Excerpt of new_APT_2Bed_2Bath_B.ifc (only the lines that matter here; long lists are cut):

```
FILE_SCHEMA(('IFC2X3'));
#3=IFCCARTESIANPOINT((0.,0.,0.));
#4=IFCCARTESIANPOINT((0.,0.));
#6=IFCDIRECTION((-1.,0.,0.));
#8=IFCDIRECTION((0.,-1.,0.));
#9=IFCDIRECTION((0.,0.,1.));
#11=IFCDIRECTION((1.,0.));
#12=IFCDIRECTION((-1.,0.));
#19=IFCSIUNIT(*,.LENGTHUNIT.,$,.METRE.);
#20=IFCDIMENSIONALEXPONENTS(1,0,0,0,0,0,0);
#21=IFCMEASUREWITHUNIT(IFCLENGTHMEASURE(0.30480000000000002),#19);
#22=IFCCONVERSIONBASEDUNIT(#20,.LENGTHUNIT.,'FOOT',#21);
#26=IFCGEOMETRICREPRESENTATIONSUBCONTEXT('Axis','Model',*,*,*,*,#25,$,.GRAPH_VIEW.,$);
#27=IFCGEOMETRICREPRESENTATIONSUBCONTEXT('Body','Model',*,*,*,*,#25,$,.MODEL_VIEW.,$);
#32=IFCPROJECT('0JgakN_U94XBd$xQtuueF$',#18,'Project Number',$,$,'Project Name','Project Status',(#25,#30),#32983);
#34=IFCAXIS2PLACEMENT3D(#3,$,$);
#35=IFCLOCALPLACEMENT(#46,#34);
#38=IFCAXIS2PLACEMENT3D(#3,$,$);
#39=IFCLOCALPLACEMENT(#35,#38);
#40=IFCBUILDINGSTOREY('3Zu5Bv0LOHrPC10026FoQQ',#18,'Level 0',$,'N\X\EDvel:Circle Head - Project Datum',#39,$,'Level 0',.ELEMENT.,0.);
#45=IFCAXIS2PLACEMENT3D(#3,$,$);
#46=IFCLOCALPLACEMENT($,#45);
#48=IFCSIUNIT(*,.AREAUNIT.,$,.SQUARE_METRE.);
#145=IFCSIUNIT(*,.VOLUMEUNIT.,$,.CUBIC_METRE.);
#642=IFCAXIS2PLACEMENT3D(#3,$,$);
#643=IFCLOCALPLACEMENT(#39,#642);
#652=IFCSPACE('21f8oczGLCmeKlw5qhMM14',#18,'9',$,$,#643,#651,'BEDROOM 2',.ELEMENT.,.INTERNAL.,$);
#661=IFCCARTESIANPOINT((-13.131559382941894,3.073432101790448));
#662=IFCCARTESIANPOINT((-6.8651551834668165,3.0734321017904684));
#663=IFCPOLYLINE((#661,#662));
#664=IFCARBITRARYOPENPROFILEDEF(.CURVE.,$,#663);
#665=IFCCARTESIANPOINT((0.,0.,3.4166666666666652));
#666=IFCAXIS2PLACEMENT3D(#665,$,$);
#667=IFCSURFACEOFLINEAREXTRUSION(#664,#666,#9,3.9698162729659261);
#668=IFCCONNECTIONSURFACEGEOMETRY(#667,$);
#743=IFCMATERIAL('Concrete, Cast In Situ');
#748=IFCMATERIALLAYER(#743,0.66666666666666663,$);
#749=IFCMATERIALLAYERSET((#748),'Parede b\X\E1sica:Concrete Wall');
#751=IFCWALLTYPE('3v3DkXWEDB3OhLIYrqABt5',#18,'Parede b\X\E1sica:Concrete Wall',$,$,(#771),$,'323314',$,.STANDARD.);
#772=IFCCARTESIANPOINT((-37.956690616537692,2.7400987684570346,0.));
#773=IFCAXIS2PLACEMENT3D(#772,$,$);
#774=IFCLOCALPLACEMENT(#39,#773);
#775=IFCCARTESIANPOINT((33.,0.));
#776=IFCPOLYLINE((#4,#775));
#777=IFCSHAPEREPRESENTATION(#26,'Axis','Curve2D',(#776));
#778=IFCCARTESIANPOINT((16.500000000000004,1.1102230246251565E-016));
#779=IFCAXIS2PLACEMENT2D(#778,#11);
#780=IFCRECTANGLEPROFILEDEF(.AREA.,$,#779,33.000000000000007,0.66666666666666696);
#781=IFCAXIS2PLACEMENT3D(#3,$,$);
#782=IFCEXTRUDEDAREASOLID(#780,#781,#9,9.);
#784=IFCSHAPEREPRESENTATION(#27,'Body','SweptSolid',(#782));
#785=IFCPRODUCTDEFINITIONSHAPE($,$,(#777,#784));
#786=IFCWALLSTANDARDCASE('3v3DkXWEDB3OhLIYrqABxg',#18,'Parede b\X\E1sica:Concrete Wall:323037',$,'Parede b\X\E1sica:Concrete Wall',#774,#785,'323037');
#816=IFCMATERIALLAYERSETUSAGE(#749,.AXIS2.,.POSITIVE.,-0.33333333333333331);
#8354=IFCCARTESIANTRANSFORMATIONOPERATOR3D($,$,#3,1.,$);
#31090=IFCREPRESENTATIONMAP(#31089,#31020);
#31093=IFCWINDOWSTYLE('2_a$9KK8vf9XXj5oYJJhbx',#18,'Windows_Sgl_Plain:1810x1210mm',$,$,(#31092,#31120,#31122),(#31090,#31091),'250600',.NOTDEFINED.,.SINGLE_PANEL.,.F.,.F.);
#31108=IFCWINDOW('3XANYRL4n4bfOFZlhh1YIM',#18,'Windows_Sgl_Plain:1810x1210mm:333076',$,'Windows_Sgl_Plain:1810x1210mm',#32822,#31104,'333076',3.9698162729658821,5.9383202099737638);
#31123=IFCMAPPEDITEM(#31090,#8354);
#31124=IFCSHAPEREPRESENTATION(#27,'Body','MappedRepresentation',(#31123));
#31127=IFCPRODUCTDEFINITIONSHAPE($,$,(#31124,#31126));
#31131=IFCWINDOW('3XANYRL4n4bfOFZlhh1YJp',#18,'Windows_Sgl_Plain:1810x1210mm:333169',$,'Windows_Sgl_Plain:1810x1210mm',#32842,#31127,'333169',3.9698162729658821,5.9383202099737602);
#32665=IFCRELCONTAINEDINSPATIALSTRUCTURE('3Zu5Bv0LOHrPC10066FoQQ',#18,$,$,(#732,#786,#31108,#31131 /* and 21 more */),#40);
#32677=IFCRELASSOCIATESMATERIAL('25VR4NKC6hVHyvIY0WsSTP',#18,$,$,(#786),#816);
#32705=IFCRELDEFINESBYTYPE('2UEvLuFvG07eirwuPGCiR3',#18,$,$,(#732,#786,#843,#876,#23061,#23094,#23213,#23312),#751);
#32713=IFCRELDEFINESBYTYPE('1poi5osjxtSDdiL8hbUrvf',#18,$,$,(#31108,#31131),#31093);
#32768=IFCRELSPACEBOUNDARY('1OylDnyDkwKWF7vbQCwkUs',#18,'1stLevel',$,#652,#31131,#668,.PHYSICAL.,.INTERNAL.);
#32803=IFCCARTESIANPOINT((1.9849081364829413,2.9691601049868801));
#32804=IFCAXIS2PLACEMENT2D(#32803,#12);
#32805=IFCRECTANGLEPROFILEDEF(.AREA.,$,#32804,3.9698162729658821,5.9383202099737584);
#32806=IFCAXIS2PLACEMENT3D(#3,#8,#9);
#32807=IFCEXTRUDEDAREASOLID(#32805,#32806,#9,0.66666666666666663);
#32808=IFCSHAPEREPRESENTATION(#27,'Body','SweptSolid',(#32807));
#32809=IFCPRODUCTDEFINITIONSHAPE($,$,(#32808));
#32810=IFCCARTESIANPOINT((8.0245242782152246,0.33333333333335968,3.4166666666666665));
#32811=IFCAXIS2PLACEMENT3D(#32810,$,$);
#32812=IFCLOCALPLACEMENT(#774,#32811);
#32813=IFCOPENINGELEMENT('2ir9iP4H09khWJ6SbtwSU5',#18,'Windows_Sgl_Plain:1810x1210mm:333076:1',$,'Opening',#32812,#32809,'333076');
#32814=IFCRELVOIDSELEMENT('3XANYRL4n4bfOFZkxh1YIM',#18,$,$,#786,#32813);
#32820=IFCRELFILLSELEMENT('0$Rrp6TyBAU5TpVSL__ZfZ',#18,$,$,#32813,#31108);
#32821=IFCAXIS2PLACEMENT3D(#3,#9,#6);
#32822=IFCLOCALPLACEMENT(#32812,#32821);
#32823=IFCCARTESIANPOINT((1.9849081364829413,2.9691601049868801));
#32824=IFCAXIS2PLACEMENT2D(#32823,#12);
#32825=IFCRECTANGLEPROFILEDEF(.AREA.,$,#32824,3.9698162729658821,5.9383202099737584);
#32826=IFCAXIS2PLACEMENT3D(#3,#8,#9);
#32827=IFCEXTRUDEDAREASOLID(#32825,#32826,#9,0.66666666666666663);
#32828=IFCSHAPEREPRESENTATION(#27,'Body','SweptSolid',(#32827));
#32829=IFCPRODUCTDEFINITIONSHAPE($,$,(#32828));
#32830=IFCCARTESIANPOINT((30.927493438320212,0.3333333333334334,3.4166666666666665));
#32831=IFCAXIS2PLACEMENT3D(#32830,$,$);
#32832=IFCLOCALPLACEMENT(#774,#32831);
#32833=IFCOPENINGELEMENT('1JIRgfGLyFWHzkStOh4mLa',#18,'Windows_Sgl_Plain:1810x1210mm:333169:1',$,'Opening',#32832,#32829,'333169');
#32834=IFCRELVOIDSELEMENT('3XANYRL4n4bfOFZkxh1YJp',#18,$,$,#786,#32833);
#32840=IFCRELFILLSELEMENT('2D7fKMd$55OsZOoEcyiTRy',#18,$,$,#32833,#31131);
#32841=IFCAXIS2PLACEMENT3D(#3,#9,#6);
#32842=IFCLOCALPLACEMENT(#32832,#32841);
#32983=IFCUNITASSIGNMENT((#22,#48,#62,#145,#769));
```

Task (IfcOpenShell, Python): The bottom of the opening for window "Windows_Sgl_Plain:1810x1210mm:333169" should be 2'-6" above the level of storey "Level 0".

```python
import numpy as np
import ifcopenshell
import ifcopenshell.api.geometry
import ifcopenshell.geom
import ifcopenshell.util.element
import ifcopenshell.util.placement
import ifcopenshell.util.shape
import ifcopenshell.util.unit

model = ifcopenshell.open("new_APT_2Bed_2Bath_B.ifc")
unit_scale = ifcopenshell.util.unit.calculate_unit_scale(model)

window = model.by_guid("3XANYRL4n4bfOFZlhh1YJp")
opening = window.FillsVoids[0].RelatingOpeningElement
storey = ifcopenshell.util.element.get_container(window, ifc_class="IfcBuildingStorey")
level = ifcopenshell.util.placement.get_local_placement(storey.ObjectPlacement)[2, 3]

# The opening's origin need not be at the sill, so measure its lowest point.
shape = ifcopenshell.geom.create_shape(ifcopenshell.geom.settings(), opening)
bottom = ifcopenshell.util.shape.get_shape_bottom_elevation(shape, shape.geometry) / unit_scale
dz = level + 30 * 0.0254 / unit_scale - bottom

shift = np.array([0.0, 0.0, dz])
# The window is placed relative to its opening, so it follows when the opening moves.
matrix = ifcopenshell.util.placement.get_local_placement(opening.ObjectPlacement)
matrix[:3, 3] += shift
ifcopenshell.api.geometry.edit_object_placement(
    model, product=opening, matrix=matrix, is_si=False, should_transform_children=True
)

# Space boundary surfaces are stored in each space's coordinates; move them too.
for rel in window.ProvidesBoundaries:
    if not rel.ConnectionGeometry:
        continue
    surface = rel.ConnectionGeometry.SurfaceOnRelatingElement
    space_matrix = ifcopenshell.util.placement.get_local_placement(rel.RelatingSpace.ObjectPlacement)
    point = np.array(surface.Position.Location.Coordinates) + space_matrix[:3, :3].T @ shift
    surface.Position = model.createIfcAxis2Placement3D(
        model.createIfcCartesianPoint(point.tolist()), surface.Position.Axis, surface.Position.RefDirection
    )

print(f"moved by {dz * unit_scale:+.3f} m")

model.write("new_APT_2Bed_2Bath_B_edited.ifc")
```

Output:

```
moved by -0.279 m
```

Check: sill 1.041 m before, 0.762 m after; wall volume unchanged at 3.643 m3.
